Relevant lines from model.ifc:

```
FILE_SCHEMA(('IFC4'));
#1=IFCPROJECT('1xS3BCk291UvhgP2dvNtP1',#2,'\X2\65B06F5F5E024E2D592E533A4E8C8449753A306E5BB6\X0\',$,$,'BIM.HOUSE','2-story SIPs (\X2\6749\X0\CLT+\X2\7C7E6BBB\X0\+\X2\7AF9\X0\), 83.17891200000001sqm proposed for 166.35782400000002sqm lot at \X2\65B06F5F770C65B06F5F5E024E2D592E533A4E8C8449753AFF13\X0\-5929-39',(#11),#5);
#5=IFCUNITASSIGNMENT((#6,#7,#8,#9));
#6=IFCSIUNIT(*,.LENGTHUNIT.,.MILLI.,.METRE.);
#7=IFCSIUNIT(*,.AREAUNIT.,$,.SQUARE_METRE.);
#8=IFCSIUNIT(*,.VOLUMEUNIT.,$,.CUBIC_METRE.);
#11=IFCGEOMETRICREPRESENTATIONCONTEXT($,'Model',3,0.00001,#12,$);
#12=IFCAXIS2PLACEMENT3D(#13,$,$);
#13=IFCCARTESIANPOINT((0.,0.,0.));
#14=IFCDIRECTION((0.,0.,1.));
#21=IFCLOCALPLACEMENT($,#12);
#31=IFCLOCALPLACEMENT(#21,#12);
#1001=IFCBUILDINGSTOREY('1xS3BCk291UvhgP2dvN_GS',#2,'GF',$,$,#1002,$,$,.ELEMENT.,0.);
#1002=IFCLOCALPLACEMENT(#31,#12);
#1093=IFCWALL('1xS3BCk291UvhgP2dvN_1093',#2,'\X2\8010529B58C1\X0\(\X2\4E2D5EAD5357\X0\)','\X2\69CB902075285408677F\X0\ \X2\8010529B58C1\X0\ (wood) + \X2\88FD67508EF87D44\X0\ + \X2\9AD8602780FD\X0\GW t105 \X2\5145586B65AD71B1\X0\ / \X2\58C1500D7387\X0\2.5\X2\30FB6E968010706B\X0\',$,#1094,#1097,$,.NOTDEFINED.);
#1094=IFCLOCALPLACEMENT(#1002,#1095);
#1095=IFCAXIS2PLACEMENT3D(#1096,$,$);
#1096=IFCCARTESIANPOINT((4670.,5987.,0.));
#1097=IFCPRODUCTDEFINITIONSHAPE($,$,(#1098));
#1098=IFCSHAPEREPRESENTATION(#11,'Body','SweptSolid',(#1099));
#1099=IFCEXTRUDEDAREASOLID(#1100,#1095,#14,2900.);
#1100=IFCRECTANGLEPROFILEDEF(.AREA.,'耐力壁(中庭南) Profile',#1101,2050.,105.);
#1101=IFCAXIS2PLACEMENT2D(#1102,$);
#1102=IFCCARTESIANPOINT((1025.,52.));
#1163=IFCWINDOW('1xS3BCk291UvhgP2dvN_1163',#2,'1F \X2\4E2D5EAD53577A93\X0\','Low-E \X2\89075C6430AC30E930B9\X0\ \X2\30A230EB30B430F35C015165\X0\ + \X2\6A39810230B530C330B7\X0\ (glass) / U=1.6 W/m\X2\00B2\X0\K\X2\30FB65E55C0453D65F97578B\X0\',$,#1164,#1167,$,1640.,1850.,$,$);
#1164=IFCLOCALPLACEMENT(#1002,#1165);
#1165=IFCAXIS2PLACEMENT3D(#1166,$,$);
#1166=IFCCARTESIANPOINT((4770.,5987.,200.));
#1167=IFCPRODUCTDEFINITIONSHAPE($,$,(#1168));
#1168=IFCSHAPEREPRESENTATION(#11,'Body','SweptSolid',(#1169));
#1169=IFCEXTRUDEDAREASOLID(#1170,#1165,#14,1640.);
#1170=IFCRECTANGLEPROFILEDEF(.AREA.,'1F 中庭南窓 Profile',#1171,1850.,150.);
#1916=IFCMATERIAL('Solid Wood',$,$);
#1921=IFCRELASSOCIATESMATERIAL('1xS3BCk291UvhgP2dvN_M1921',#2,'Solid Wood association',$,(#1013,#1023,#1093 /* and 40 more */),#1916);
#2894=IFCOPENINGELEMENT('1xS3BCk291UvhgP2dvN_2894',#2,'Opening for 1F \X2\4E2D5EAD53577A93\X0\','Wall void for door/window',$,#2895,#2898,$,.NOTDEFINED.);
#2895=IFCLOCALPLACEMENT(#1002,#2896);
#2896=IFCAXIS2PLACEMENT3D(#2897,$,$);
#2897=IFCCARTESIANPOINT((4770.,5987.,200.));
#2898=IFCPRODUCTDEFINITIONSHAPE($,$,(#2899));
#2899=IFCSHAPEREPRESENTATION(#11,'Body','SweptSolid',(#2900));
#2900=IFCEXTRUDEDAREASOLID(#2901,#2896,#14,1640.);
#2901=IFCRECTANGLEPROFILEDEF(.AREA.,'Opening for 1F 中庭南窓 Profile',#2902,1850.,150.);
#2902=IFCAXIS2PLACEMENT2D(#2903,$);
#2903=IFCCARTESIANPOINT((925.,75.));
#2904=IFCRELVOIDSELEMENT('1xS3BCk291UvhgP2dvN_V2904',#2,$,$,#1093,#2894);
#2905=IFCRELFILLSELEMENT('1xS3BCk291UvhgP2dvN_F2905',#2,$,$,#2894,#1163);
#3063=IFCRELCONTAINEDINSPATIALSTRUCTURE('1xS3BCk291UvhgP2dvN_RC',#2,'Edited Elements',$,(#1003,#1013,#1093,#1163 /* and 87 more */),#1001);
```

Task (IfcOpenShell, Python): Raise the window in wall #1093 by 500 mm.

```python
import numpy as np
import ifcopenshell
import ifcopenshell.api.geometry
import ifcopenshell.util.placement
import ifcopenshell.util.unit

model = ifcopenshell.open("model.ifc")
unit_scale = ifcopenshell.util.unit.calculate_unit_scale(model)

window = model.by_id(1163)
opening = window.FillsVoids[0].RelatingOpeningElement
dz = 0.5 / unit_scale

shift = np.array([0.0, 0.0, dz])
# The window is not placed relative to its opening, so move both.
for product in (opening, window):
    matrix = ifcopenshell.util.placement.get_local_placement(product.ObjectPlacement)
    matrix[:3, 3] += shift
    ifcopenshell.api.geometry.edit_object_placement(model, product=product, matrix=matrix, is_si=False)

print(f"moved by {dz * unit_scale:+.3f} m")

model.write("model_rev.ifc")
```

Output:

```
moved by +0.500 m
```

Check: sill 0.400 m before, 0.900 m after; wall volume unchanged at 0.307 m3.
